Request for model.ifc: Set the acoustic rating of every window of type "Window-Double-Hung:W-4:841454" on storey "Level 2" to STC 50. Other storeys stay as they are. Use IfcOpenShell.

First a look at what the model holds.

```python
import ifcopenshell
import ifcopenshell.util.element

model = ifcopenshell.open("model.ifc")
print(model.schema)
storey = next(s for s in model.by_type("IfcBuildingStorey") if s.Name == "Level 2")
windows = [e for e in ifcopenshell.util.element.get_decomposition(storey) if e.is_a("IfcWindow")]
seen = {}
for e in windows:
    element_type = ifcopenshell.util.element.get_type(e)
    key = (element_type.Name if element_type != e and element_type else None, ifcopenshell.util.element.get_pset(e, "Pset_WindowCommon", "AcousticRating"))
    seen[key] = seen.get(key, 0) + 1
for (name, value), count in sorted(seen.items(), key=str):
    print(count, "x", name, "|", value)
```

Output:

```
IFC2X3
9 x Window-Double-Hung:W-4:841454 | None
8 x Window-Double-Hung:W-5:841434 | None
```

```python
import ifcopenshell
import ifcopenshell.api.pset
import ifcopenshell.util.element

model = ifcopenshell.open("model.ifc")

storey = next(s for s in model.by_type("IfcBuildingStorey") if s.Name == "Level 2")
windows = [e for e in ifcopenshell.util.element.get_decomposition(storey) if e.is_a("IfcWindow")]

count = 0
for e in windows:
    element_type = ifcopenshell.util.element.get_type(e)
    if element_type in (None, e) or element_type.Name != "Window-Double-Hung:W-4:841454":
        continue
    # add_pset returns the element's existing set when there is one.
    pset = ifcopenshell.api.pset.add_pset(model, product=e, name="Pset_WindowCommon")
    ifcopenshell.api.pset.edit_pset(model, pset=pset, properties={"AcousticRating": "STC 50"})
    count += 1

print(count, "windows updated")

model.write("model-out.ifc")
```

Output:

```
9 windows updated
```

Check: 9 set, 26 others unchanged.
